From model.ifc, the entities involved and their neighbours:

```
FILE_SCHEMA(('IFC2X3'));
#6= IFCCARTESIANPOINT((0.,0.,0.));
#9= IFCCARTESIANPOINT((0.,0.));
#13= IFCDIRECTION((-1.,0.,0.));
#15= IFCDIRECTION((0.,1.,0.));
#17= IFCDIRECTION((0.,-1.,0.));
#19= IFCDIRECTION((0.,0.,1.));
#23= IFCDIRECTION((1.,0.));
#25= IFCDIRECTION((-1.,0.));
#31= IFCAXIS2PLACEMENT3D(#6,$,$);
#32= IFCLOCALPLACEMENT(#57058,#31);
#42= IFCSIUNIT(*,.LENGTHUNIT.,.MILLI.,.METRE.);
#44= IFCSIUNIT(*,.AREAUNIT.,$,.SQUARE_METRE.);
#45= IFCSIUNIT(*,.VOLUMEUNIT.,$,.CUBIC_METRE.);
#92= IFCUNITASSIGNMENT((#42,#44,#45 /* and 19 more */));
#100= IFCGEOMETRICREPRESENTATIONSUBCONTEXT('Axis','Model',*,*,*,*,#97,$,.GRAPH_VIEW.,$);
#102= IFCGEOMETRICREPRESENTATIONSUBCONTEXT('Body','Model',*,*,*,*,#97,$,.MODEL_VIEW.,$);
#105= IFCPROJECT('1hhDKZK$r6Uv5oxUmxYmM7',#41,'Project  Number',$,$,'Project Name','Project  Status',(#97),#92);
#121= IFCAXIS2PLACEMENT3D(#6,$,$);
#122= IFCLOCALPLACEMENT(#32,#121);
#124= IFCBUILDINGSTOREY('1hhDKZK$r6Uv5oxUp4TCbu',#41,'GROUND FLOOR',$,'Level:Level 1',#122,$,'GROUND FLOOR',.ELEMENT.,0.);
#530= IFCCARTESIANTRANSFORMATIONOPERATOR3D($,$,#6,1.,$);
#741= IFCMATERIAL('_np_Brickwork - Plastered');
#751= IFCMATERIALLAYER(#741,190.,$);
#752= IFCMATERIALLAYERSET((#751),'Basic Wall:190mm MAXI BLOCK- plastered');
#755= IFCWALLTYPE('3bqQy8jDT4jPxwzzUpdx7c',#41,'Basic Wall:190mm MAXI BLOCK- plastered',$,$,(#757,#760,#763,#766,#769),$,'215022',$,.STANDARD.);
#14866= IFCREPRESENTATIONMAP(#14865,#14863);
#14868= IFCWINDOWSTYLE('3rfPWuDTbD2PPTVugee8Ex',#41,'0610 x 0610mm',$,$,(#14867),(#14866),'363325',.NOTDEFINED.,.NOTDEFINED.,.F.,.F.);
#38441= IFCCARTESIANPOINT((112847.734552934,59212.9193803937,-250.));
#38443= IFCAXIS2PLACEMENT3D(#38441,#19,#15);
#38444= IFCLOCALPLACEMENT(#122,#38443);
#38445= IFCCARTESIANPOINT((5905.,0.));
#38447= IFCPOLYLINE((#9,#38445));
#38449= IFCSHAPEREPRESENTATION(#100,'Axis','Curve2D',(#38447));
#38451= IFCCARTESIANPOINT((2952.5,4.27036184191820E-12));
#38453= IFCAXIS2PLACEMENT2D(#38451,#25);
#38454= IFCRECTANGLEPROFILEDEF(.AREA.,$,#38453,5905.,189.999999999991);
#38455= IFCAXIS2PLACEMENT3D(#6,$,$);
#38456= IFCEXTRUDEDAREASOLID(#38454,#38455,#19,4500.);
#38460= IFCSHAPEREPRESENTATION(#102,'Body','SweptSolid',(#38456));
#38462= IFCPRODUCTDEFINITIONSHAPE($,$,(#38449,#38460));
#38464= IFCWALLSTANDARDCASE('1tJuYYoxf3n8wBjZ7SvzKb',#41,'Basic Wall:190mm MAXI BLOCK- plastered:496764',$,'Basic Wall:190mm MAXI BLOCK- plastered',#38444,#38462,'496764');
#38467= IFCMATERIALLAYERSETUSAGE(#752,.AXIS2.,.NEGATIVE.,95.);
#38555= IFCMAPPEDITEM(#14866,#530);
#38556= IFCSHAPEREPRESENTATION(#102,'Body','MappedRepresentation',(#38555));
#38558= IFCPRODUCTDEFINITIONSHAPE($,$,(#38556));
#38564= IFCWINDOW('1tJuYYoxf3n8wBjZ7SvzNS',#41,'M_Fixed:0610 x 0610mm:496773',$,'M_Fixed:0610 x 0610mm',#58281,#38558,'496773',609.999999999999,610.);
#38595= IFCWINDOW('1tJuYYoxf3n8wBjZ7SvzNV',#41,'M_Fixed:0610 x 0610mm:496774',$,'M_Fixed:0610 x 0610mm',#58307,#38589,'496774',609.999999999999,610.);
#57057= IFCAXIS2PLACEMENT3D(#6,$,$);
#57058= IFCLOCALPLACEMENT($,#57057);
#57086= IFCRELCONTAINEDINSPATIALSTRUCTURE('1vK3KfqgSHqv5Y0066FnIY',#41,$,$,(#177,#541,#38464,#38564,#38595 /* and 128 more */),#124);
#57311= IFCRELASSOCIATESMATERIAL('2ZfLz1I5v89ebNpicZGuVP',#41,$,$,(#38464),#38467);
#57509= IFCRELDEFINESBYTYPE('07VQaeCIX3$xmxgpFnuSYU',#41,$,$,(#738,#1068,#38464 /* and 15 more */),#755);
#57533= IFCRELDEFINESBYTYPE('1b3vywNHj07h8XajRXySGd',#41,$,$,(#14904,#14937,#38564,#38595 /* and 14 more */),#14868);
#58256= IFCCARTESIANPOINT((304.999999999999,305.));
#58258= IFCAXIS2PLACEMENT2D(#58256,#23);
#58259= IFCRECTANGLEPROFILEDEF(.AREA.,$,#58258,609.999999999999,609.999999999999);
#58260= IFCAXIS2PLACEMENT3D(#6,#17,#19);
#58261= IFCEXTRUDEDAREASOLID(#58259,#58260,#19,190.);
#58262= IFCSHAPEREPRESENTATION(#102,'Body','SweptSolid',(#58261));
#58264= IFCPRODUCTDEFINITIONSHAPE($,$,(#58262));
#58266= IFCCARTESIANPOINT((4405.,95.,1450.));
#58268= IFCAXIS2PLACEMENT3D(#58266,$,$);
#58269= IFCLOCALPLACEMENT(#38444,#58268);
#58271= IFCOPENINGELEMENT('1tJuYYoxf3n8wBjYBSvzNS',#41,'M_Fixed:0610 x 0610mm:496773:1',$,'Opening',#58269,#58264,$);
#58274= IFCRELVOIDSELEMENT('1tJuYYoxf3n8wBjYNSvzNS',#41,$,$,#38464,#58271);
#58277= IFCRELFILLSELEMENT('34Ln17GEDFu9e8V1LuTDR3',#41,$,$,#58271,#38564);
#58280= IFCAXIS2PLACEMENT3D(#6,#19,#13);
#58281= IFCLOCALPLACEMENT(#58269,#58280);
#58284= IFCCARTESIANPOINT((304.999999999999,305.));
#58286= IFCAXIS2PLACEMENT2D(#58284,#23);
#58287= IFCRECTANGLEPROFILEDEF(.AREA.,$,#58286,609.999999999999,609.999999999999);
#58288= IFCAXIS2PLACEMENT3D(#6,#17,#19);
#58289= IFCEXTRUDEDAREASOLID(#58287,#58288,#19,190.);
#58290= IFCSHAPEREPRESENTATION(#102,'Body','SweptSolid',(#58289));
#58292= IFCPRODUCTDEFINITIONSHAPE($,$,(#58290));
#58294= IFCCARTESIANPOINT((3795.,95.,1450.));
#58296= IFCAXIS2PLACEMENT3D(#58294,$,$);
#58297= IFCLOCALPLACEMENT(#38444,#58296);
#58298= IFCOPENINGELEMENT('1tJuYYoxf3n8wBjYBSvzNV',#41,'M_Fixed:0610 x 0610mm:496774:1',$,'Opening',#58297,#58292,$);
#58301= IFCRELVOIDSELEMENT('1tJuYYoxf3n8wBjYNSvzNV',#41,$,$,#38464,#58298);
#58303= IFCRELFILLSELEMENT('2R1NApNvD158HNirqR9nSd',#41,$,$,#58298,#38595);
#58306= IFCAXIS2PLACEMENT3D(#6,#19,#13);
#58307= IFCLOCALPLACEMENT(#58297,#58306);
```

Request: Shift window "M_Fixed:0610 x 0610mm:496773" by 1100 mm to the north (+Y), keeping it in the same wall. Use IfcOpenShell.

```python
import ifcopenshell
import ifcopenshell.api.geometry
import ifcopenshell.util.placement

model = ifcopenshell.open("model.ifc")

window = model.by_guid("1tJuYYoxf3n8wBjZ7SvzNS")
opening = window.FillsVoids[0].RelatingOpeningElement
wall = opening.VoidsElements[0].RelatingBuildingElement

wall_matrix = ifcopenshell.util.placement.get_local_placement(wall.ObjectPlacement)
shift = wall_matrix[:3, 0] * 1100.0
before = ifcopenshell.util.placement.get_local_placement(window.ObjectPlacement)[:3, 3].copy()

# The window is placed relative to its opening, so it follows when the opening moves.
matrix = ifcopenshell.util.placement.get_local_placement(opening.ObjectPlacement)
matrix[:3, 3] += shift
ifcopenshell.api.geometry.edit_object_placement(
    model, product=opening, matrix=matrix, is_si=False, should_transform_children=True
)

after = ifcopenshell.util.placement.get_local_placement(window.ObjectPlacement)[:3, 3]
print("window moved by", (after - before).round(3) + 0.0)

model.write("model_updated.ifc")
```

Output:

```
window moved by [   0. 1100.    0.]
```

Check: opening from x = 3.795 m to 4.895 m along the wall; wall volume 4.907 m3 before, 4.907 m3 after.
